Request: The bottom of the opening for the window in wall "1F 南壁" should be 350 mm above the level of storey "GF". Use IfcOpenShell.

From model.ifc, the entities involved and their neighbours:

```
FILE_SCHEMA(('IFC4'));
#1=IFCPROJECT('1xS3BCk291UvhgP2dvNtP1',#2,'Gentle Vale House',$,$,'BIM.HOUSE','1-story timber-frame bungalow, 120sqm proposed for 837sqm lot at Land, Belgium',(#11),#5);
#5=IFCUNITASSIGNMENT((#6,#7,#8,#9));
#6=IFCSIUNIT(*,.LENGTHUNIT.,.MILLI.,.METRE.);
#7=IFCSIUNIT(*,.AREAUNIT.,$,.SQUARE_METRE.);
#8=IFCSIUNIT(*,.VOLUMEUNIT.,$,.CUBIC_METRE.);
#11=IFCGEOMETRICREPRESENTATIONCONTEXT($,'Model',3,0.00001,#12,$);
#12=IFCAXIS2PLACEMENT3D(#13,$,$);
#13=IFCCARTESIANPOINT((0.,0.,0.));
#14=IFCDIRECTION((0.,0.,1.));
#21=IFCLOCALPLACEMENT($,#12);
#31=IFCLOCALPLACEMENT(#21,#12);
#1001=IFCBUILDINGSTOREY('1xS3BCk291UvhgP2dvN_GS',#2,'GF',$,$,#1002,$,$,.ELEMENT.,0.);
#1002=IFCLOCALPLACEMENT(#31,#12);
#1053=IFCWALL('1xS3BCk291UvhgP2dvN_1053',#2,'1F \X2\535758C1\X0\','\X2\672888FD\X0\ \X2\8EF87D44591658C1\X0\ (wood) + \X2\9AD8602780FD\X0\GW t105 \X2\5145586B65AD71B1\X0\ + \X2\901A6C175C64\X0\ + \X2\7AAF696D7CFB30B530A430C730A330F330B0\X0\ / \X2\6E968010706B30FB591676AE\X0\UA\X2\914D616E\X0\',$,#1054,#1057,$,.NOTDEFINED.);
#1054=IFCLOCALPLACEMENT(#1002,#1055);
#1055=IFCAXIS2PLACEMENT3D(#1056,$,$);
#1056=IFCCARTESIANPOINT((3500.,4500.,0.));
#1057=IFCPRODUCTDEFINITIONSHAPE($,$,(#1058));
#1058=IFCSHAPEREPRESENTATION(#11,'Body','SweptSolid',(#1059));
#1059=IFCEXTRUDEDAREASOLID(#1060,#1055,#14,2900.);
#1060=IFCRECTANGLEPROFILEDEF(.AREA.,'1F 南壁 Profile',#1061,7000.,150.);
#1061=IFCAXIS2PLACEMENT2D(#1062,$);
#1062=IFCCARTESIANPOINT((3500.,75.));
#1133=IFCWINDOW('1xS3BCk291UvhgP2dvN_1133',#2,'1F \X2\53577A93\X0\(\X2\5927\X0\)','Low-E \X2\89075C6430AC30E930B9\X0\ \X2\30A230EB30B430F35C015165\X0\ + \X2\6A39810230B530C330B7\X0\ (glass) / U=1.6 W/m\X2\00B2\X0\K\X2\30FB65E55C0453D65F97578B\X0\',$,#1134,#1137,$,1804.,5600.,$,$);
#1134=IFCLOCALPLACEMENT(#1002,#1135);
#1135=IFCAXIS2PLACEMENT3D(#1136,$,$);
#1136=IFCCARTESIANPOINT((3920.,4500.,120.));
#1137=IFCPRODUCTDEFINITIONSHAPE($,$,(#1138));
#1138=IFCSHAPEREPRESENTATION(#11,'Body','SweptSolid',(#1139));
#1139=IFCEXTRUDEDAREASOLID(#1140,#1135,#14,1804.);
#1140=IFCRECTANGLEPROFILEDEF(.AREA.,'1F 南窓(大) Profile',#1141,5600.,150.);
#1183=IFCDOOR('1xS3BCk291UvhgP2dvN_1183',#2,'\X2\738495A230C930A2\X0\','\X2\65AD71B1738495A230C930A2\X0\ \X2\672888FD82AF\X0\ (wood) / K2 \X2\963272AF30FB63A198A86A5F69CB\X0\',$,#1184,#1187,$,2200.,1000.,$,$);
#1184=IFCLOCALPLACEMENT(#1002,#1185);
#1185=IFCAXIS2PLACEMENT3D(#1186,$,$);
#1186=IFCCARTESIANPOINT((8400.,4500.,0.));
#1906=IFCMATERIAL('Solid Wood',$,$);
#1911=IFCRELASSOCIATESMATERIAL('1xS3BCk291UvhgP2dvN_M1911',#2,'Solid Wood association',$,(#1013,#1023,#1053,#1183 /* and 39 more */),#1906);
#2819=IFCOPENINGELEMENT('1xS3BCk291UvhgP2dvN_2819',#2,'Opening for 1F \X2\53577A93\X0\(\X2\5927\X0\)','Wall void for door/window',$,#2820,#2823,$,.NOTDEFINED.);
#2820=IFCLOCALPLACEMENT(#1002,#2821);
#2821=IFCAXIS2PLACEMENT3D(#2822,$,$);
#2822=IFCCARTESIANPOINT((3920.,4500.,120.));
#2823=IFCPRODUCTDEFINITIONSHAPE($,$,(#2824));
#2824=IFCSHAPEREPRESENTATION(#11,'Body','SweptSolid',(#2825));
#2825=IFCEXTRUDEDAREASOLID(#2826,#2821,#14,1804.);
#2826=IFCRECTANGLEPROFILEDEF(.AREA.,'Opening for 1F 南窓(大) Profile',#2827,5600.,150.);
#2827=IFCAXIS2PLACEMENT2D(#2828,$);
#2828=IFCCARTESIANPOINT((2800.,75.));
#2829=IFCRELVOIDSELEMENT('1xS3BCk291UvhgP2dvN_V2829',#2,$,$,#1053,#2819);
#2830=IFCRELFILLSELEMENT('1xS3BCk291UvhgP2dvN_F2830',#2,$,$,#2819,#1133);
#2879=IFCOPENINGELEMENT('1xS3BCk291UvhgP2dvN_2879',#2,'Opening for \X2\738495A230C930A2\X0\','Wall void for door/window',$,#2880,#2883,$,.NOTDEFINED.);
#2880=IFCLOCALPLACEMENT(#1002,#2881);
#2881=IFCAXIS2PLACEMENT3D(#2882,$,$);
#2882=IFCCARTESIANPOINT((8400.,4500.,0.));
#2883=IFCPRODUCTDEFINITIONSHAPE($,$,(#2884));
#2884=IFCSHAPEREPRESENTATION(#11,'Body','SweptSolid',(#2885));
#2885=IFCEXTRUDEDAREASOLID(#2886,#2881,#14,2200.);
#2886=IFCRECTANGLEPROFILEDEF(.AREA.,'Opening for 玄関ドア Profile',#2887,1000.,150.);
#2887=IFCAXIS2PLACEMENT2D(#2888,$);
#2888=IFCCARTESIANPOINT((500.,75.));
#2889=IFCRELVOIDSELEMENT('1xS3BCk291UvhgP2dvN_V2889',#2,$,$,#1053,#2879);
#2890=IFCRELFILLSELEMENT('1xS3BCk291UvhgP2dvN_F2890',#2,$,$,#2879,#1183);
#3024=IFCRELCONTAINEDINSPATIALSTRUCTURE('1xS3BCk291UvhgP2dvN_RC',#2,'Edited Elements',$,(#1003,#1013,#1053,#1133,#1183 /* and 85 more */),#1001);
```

```python
import numpy as np
import ifcopenshell
import ifcopenshell.api.geometry
import ifcopenshell.geom
import ifcopenshell.util.element
import ifcopenshell.util.placement
import ifcopenshell.util.shape
import ifcopenshell.util.unit

model = ifcopenshell.open("model.ifc")
unit_scale = ifcopenshell.util.unit.calculate_unit_scale(model)

window = model.by_id(1133)
opening = window.FillsVoids[0].RelatingOpeningElement
storey = ifcopenshell.util.element.get_container(window, ifc_class="IfcBuildingStorey")
level = ifcopenshell.util.placement.get_local_placement(storey.ObjectPlacement)[2, 3]

# The opening's origin need not be at the sill, so measure its lowest point.
shape = ifcopenshell.geom.create_shape(ifcopenshell.geom.settings(), opening)
bottom = ifcopenshell.util.shape.get_shape_bottom_elevation(shape, shape.geometry) / unit_scale
dz = level + 350.0 - bottom

shift = np.array([0.0, 0.0, dz])
# The window is not placed relative to its opening, so move both.
for product in (opening, window):
    matrix = ifcopenshell.util.placement.get_local_placement(product.ObjectPlacement)
    matrix[:3, 3] += shift
    ifcopenshell.api.geometry.edit_object_placement(model, product=product, matrix=matrix, is_si=False)

print(f"moved by {dz * unit_scale:+.3f} m")

model.write("model_rev.ifc")
```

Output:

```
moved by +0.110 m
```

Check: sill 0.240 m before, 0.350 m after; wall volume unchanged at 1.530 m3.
